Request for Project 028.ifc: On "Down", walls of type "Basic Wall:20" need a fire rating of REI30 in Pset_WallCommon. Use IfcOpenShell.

First a look at what the model holds.

```python
import ifcopenshell
import ifcopenshell.util.element

model = ifcopenshell.open("Project 028.ifc")
print(model.schema)
storey = next(s for s in model.by_type("IfcBuildingStorey") if s.Name == "Down")
walls = [e for e in ifcopenshell.util.element.get_decomposition(storey) if e.is_a("IfcWall")]
seen = {}
for e in walls:
    element_type = ifcopenshell.util.element.get_type(e)
    key = (element_type.Name if element_type != e and element_type else None, ifcopenshell.util.element.get_pset(e, "Pset_WallCommon", "FireRating"))
    seen[key] = seen.get(key, 0) + 1
for (name, value), count in sorted(seen.items(), key=str):
    print(count, "x", name, "|", value)
```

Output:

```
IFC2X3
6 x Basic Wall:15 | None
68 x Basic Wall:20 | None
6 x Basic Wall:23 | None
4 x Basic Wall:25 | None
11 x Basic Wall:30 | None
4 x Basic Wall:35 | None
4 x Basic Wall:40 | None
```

```python
import ifcopenshell
import ifcopenshell.api.pset
import ifcopenshell.util.element

model = ifcopenshell.open("Project 028.ifc")

storey = next(s for s in model.by_type("IfcBuildingStorey") if s.Name == "Down")
walls = [e for e in ifcopenshell.util.element.get_decomposition(storey) if e.is_a("IfcWall")]

count = 0
for e in walls:
    element_type = ifcopenshell.util.element.get_type(e)
    if element_type in (None, e) or element_type.Name != "Basic Wall:20":
        continue
    # add_pset returns the element's existing set when there is one.
    pset = ifcopenshell.api.pset.add_pset(model, product=e, name="Pset_WallCommon")
    ifcopenshell.api.pset.edit_pset(model, pset=pset, properties={"FireRating": "REI30"})
    count += 1

print(count, "walls updated")

model.write("Project 028_updated.ifc")
```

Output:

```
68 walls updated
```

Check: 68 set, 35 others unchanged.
